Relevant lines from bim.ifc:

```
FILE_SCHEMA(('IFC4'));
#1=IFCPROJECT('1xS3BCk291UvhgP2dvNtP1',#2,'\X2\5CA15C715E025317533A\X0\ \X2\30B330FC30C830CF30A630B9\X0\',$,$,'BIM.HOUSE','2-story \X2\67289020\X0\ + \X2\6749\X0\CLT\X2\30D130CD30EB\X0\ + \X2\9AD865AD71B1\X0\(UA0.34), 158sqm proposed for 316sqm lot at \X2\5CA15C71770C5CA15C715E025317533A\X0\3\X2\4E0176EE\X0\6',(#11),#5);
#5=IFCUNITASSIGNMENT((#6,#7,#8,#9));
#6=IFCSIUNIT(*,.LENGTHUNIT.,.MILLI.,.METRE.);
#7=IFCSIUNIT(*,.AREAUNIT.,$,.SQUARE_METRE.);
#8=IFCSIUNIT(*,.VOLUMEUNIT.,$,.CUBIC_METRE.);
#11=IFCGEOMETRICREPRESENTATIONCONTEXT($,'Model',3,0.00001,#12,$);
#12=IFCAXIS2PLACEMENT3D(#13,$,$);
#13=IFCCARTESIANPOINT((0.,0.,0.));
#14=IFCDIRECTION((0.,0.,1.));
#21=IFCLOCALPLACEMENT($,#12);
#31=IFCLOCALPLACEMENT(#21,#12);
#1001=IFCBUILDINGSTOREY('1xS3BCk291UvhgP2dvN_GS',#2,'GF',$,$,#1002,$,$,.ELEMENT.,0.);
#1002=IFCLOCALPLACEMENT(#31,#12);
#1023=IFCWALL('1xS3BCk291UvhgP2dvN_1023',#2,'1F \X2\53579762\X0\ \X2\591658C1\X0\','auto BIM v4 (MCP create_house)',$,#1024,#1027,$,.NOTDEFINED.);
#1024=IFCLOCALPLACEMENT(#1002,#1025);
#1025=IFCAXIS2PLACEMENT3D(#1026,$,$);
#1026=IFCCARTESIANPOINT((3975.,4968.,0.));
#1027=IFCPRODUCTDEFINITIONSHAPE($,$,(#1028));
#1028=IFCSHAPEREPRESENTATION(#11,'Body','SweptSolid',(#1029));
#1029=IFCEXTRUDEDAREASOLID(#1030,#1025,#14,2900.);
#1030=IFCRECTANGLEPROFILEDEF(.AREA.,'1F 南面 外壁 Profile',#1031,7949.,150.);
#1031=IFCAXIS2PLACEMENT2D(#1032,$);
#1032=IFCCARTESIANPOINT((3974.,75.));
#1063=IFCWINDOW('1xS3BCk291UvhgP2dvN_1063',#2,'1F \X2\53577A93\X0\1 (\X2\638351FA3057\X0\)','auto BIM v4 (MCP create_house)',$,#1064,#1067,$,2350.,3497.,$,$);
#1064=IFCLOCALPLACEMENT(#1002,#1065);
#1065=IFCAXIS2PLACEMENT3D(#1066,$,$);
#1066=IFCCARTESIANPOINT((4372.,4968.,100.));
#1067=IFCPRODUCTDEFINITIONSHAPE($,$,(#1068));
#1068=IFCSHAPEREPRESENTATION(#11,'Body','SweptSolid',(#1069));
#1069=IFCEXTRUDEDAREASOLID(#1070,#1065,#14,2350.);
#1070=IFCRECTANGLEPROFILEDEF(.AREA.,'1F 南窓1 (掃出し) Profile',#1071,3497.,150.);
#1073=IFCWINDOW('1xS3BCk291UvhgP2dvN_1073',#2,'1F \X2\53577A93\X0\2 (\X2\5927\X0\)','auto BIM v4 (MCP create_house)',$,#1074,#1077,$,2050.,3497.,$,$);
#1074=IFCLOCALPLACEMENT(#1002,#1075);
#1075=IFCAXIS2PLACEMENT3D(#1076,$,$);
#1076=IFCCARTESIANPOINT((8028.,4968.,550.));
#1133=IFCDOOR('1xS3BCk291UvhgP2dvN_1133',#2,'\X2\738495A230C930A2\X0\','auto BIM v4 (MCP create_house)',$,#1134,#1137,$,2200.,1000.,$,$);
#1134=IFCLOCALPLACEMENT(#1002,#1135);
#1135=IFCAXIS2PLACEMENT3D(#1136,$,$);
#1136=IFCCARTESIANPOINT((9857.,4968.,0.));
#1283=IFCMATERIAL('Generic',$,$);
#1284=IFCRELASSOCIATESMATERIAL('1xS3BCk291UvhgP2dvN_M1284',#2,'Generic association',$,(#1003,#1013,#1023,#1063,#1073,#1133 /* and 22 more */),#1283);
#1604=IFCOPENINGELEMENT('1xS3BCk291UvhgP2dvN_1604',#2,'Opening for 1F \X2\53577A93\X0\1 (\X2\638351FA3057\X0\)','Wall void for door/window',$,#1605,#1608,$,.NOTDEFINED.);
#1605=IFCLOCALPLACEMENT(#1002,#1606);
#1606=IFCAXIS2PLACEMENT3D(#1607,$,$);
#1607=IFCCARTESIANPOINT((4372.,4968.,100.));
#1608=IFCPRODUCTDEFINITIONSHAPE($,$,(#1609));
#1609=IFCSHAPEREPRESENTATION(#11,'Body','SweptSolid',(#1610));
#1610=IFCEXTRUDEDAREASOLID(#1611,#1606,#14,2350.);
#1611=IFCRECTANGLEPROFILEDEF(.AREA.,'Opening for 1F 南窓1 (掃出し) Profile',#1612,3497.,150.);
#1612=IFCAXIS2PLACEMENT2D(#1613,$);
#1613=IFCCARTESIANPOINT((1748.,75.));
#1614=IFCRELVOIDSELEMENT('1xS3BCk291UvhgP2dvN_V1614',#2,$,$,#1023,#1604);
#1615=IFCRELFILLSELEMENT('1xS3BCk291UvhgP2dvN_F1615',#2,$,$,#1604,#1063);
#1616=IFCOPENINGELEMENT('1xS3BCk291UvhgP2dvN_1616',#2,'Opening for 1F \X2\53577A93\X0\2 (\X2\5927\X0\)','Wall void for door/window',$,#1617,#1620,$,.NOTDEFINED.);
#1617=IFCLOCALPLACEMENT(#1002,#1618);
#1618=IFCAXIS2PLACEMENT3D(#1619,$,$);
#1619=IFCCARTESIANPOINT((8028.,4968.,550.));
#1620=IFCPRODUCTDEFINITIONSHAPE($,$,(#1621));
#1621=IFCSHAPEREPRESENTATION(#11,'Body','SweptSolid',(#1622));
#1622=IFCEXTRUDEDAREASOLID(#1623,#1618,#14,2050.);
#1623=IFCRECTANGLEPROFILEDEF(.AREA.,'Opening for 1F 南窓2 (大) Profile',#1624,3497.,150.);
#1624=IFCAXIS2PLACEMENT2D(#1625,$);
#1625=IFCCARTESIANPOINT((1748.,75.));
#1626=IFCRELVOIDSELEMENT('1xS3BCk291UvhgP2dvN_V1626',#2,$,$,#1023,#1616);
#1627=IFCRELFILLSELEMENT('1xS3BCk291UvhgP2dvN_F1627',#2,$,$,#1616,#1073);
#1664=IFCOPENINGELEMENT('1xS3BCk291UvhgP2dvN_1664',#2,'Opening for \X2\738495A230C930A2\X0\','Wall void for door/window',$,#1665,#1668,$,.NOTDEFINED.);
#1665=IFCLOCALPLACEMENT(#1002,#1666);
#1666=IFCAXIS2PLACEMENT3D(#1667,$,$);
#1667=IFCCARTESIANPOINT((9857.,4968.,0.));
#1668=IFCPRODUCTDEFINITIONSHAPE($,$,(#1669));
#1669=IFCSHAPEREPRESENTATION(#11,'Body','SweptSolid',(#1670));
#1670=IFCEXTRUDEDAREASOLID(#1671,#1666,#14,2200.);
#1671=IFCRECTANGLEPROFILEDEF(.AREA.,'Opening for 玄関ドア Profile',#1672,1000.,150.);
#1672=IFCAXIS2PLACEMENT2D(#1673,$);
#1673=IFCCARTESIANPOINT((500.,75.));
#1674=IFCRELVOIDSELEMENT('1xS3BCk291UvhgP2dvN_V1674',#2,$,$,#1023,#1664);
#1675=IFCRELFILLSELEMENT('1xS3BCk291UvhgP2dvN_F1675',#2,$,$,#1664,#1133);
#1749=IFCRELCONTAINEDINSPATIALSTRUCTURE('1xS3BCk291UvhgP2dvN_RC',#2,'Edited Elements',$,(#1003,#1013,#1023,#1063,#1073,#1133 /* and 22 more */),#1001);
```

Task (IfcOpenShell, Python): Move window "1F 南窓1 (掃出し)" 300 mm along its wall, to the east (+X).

```python
import ifcopenshell
import ifcopenshell.api.geometry
import ifcopenshell.util.placement
import ifcopenshell.util.unit

model = ifcopenshell.open("bim.ifc")
unit_scale = ifcopenshell.util.unit.calculate_unit_scale(model)

window = model.by_guid("1xS3BCk291UvhgP2dvN_1063")
opening = window.FillsVoids[0].RelatingOpeningElement
wall = opening.VoidsElements[0].RelatingBuildingElement

wall_matrix = ifcopenshell.util.placement.get_local_placement(wall.ObjectPlacement)
shift = wall_matrix[:3, 0] * 0.3 / unit_scale
before = ifcopenshell.util.placement.get_local_placement(window.ObjectPlacement)[:3, 3].copy()

# The window is not placed relative to its opening, so move both.
for product in (opening, window):
    matrix = ifcopenshell.util.placement.get_local_placement(product.ObjectPlacement)
    matrix[:3, 3] += shift
    ifcopenshell.api.geometry.edit_object_placement(model, product=product, matrix=matrix, is_si=False)

after = ifcopenshell.util.placement.get_local_placement(window.ObjectPlacement)[:3, 3]
print("window moved by", (after - before).round(3) + 0.0)

model.write("bim_rev.ifc")
```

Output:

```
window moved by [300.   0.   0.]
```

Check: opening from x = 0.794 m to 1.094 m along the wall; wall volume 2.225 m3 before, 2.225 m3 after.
